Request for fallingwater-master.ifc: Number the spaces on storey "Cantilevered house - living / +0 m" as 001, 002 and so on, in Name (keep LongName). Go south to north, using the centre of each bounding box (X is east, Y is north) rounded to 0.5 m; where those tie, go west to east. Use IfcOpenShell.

First a look at what the model holds.

```python
import ifcopenshell
import ifcopenshell.util.element
import ifcopenshell.util.placement

model = ifcopenshell.open("fallingwater-master.ifc")
print(model.schema)
storey = next(s for s in model.by_type("IfcBuildingStorey") if s.Name == "Cantilevered house - living / +0 m")
spaces = [e for e in ifcopenshell.util.element.get_decomposition(storey) if e.is_a("IfcSpace")]
for e in sorted(spaces, key=lambda e: e.id()):
    origin = ifcopenshell.util.placement.get_local_placement(e.ObjectPlacement)[:3, 3]
    print(e.id(), e.Name, e.LongName, origin.round(2) + 0.0, sep=" | ")
```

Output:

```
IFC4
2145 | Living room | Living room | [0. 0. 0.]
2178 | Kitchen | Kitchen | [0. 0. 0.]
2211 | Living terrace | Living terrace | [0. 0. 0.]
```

```python
import ifcopenshell
import ifcopenshell.geom
import ifcopenshell.util.element
import ifcopenshell.util.shape

model = ifcopenshell.open("fallingwater-master.ifc")
settings = ifcopenshell.geom.settings()
settings.set("use-world-coords", True)


def centre(element):
    shape = ifcopenshell.geom.create_shape(settings, element)
    return ifcopenshell.util.shape.get_bbox_centroid(shape.geometry)


storey = next(s for s in model.by_type("IfcBuildingStorey") if s.Name == "Cantilevered house - living / +0 m")
spaces = [e for e in ifcopenshell.util.element.get_decomposition(storey) if e.is_a("IfcSpace")]

# Insertion points can sit at a corner or the storey origin, so sort by the geometry (in metres).
centres = {e: centre(e) for e in spaces}
spaces.sort(key=lambda e: (round(centres[e][1] / 0.5), centres[e][0]))

for i, e in enumerate(spaces, start=1):
    number = f"0{i:02d}"
    e.Name = number
    print(e.id(), number)

model.write("fallingwater-master_v2.ifc")
```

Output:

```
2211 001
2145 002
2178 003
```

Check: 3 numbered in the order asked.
